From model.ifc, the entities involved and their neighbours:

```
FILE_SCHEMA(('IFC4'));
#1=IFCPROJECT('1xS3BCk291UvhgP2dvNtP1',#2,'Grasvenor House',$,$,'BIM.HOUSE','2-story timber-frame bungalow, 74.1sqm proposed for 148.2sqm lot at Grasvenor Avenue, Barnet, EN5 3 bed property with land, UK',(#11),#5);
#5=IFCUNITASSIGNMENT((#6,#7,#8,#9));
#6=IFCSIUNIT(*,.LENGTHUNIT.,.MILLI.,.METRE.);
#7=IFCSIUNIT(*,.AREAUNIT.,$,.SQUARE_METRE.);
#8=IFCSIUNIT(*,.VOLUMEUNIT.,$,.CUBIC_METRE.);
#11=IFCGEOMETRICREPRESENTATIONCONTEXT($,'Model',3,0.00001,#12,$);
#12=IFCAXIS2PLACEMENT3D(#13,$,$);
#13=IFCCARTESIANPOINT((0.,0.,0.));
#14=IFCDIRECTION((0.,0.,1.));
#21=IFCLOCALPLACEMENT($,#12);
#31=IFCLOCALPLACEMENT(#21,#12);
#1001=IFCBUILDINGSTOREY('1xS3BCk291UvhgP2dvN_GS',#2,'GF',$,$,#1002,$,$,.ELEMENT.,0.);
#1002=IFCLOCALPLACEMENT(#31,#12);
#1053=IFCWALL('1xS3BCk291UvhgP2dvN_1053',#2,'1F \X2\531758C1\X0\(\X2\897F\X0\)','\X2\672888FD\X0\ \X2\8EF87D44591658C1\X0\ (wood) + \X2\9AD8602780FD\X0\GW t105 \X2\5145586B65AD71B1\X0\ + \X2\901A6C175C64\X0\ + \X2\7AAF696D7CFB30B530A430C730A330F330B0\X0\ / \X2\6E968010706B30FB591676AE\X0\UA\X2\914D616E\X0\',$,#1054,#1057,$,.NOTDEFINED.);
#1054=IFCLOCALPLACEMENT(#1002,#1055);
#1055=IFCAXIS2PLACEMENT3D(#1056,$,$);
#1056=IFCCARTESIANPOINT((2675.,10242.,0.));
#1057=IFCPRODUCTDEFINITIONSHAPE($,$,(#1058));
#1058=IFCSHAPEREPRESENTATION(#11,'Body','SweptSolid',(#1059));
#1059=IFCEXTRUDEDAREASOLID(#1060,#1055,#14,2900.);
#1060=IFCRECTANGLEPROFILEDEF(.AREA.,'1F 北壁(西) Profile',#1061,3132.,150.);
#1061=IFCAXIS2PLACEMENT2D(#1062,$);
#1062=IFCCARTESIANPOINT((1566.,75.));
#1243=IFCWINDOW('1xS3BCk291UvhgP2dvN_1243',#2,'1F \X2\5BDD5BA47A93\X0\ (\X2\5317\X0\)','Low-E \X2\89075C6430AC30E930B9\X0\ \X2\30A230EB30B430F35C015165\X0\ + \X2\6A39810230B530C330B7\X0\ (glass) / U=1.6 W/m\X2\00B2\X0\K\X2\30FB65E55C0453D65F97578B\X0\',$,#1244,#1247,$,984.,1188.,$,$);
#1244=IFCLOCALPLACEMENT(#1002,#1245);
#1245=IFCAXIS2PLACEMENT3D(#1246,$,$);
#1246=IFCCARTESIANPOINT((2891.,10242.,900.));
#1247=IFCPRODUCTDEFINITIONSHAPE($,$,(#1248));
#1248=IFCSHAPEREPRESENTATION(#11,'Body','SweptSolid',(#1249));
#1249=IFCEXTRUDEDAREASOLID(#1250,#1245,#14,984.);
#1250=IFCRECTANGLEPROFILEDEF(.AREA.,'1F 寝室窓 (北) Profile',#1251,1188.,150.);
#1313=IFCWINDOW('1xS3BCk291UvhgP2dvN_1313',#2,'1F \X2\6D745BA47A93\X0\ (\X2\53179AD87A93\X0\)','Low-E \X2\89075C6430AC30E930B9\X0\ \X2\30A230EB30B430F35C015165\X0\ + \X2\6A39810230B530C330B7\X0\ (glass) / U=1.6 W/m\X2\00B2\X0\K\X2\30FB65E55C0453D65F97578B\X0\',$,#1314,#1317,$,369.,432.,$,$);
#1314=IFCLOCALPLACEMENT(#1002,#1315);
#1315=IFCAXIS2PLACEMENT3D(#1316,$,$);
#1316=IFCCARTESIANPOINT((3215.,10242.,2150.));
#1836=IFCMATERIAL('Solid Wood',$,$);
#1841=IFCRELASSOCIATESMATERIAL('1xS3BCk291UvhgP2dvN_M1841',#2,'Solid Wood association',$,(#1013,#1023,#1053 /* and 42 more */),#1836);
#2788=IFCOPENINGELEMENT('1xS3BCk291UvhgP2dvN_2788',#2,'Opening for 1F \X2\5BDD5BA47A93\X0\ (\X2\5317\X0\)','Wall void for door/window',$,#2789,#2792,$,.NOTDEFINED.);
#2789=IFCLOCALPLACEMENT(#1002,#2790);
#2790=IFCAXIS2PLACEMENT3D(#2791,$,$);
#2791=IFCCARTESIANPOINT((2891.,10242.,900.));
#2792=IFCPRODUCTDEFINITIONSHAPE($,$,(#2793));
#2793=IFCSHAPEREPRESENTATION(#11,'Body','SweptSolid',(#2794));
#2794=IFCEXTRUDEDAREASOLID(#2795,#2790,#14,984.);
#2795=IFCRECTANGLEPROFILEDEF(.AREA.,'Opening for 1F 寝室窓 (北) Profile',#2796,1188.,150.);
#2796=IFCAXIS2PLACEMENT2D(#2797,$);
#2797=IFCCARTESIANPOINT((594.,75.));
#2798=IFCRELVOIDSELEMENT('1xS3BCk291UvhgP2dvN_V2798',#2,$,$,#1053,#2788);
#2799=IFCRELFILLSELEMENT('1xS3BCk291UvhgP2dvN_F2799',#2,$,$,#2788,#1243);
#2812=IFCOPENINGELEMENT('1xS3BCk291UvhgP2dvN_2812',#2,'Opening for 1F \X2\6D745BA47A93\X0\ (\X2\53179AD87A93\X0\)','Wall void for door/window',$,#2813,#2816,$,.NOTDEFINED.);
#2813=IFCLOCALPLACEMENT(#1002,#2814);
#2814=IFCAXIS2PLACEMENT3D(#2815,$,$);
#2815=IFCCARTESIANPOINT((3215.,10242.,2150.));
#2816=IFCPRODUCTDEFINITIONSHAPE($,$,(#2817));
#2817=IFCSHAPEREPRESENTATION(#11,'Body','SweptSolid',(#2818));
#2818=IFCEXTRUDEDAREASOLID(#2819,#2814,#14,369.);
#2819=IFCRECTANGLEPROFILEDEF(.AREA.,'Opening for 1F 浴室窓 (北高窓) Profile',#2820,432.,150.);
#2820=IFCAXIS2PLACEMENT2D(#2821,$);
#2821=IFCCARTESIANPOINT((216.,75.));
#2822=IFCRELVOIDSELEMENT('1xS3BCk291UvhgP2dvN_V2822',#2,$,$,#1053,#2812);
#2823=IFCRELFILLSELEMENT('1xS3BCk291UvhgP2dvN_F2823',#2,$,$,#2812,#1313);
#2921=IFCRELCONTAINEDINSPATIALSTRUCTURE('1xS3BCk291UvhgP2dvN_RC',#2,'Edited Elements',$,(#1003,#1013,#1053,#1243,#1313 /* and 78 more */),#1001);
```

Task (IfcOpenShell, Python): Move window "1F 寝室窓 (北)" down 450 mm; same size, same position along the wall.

```python
import numpy as np
import ifcopenshell
import ifcopenshell.api.geometry
import ifcopenshell.util.placement
import ifcopenshell.util.unit

model = ifcopenshell.open("model.ifc")
unit_scale = ifcopenshell.util.unit.calculate_unit_scale(model)

window = model.by_guid("1xS3BCk291UvhgP2dvN_1243")
opening = window.FillsVoids[0].RelatingOpeningElement
dz = -450.0

shift = np.array([0.0, 0.0, dz])
# The window is not placed relative to its opening, so move both.
for product in (opening, window):
    matrix = ifcopenshell.util.placement.get_local_placement(product.ObjectPlacement)
    matrix[:3, 3] += shift
    ifcopenshell.api.geometry.edit_object_placement(model, product=product, matrix=matrix, is_si=False)

print(f"moved by {dz * unit_scale:+.3f} m")

model.write("model_v2.ifc")
```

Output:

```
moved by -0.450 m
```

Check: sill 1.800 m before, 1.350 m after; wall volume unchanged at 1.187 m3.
